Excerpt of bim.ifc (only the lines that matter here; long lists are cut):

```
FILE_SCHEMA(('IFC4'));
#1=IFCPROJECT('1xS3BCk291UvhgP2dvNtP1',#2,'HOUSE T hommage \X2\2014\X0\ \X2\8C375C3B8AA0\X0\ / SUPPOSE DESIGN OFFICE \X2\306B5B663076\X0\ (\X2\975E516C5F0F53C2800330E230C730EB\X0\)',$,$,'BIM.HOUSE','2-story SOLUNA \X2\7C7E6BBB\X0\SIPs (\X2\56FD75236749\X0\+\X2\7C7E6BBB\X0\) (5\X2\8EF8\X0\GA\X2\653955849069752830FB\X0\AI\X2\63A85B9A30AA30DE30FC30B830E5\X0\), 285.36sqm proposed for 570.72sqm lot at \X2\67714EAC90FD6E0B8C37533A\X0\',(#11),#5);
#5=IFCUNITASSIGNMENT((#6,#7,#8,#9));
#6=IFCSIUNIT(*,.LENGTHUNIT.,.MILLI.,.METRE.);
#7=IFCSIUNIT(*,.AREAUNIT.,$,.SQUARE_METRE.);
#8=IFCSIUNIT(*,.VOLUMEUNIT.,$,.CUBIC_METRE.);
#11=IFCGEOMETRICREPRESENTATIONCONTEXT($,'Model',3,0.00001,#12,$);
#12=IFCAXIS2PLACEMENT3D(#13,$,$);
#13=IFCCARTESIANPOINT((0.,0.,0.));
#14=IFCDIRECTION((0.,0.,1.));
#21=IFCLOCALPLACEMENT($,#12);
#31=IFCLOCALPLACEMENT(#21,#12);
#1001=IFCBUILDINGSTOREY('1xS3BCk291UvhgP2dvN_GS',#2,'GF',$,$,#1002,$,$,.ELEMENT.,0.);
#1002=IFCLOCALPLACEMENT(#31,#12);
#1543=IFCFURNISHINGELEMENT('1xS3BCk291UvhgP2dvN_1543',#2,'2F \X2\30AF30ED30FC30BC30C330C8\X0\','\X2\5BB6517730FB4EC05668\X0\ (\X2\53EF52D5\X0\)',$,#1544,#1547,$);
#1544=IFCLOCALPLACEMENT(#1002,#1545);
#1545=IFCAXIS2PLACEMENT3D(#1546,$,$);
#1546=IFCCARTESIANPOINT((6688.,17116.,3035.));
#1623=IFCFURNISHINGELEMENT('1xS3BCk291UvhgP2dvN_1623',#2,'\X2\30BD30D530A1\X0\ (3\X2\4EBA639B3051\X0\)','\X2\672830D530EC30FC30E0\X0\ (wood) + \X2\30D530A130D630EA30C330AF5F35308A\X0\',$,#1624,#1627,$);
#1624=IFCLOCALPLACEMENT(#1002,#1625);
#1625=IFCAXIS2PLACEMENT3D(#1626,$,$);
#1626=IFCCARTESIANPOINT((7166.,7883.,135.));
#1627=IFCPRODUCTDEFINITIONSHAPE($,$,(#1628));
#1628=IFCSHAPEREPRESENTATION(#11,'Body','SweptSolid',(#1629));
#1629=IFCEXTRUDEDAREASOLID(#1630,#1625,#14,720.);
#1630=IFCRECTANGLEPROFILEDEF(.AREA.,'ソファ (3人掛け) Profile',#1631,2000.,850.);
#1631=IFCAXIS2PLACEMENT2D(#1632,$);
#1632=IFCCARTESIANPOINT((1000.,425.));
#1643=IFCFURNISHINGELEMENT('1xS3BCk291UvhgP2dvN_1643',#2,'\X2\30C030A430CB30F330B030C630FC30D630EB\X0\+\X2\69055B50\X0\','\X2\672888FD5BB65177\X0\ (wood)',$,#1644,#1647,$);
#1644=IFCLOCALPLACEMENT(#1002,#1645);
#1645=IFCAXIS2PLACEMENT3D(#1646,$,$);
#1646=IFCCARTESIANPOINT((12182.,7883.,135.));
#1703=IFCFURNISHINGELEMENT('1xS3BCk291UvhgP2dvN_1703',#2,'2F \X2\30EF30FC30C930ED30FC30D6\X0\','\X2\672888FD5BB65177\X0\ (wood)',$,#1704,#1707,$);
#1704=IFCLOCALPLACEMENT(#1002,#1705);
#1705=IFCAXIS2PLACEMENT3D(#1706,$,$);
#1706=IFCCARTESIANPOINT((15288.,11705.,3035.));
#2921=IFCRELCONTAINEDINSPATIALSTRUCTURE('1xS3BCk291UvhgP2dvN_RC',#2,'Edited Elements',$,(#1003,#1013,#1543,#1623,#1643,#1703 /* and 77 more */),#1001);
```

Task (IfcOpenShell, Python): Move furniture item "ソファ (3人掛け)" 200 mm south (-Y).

```python
import ifcopenshell
import ifcopenshell.api.geometry
import ifcopenshell.util.placement

model = ifcopenshell.open("bim.ifc")

item = model.by_guid("1xS3BCk291UvhgP2dvN_1623")
matrix = ifcopenshell.util.placement.get_local_placement(item.ObjectPlacement)
matrix[1, 3] -= 200.0
ifcopenshell.api.geometry.edit_object_placement(model, product=item, matrix=matrix, is_si=False)

print(ifcopenshell.util.placement.get_local_placement(item.ObjectPlacement).round(3) + 0.0)

model.write("bim_edited.ifc")
```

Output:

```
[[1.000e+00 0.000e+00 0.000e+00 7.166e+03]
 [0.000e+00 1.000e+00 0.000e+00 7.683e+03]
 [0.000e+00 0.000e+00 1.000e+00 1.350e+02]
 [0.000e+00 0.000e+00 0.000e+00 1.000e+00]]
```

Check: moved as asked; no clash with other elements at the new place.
